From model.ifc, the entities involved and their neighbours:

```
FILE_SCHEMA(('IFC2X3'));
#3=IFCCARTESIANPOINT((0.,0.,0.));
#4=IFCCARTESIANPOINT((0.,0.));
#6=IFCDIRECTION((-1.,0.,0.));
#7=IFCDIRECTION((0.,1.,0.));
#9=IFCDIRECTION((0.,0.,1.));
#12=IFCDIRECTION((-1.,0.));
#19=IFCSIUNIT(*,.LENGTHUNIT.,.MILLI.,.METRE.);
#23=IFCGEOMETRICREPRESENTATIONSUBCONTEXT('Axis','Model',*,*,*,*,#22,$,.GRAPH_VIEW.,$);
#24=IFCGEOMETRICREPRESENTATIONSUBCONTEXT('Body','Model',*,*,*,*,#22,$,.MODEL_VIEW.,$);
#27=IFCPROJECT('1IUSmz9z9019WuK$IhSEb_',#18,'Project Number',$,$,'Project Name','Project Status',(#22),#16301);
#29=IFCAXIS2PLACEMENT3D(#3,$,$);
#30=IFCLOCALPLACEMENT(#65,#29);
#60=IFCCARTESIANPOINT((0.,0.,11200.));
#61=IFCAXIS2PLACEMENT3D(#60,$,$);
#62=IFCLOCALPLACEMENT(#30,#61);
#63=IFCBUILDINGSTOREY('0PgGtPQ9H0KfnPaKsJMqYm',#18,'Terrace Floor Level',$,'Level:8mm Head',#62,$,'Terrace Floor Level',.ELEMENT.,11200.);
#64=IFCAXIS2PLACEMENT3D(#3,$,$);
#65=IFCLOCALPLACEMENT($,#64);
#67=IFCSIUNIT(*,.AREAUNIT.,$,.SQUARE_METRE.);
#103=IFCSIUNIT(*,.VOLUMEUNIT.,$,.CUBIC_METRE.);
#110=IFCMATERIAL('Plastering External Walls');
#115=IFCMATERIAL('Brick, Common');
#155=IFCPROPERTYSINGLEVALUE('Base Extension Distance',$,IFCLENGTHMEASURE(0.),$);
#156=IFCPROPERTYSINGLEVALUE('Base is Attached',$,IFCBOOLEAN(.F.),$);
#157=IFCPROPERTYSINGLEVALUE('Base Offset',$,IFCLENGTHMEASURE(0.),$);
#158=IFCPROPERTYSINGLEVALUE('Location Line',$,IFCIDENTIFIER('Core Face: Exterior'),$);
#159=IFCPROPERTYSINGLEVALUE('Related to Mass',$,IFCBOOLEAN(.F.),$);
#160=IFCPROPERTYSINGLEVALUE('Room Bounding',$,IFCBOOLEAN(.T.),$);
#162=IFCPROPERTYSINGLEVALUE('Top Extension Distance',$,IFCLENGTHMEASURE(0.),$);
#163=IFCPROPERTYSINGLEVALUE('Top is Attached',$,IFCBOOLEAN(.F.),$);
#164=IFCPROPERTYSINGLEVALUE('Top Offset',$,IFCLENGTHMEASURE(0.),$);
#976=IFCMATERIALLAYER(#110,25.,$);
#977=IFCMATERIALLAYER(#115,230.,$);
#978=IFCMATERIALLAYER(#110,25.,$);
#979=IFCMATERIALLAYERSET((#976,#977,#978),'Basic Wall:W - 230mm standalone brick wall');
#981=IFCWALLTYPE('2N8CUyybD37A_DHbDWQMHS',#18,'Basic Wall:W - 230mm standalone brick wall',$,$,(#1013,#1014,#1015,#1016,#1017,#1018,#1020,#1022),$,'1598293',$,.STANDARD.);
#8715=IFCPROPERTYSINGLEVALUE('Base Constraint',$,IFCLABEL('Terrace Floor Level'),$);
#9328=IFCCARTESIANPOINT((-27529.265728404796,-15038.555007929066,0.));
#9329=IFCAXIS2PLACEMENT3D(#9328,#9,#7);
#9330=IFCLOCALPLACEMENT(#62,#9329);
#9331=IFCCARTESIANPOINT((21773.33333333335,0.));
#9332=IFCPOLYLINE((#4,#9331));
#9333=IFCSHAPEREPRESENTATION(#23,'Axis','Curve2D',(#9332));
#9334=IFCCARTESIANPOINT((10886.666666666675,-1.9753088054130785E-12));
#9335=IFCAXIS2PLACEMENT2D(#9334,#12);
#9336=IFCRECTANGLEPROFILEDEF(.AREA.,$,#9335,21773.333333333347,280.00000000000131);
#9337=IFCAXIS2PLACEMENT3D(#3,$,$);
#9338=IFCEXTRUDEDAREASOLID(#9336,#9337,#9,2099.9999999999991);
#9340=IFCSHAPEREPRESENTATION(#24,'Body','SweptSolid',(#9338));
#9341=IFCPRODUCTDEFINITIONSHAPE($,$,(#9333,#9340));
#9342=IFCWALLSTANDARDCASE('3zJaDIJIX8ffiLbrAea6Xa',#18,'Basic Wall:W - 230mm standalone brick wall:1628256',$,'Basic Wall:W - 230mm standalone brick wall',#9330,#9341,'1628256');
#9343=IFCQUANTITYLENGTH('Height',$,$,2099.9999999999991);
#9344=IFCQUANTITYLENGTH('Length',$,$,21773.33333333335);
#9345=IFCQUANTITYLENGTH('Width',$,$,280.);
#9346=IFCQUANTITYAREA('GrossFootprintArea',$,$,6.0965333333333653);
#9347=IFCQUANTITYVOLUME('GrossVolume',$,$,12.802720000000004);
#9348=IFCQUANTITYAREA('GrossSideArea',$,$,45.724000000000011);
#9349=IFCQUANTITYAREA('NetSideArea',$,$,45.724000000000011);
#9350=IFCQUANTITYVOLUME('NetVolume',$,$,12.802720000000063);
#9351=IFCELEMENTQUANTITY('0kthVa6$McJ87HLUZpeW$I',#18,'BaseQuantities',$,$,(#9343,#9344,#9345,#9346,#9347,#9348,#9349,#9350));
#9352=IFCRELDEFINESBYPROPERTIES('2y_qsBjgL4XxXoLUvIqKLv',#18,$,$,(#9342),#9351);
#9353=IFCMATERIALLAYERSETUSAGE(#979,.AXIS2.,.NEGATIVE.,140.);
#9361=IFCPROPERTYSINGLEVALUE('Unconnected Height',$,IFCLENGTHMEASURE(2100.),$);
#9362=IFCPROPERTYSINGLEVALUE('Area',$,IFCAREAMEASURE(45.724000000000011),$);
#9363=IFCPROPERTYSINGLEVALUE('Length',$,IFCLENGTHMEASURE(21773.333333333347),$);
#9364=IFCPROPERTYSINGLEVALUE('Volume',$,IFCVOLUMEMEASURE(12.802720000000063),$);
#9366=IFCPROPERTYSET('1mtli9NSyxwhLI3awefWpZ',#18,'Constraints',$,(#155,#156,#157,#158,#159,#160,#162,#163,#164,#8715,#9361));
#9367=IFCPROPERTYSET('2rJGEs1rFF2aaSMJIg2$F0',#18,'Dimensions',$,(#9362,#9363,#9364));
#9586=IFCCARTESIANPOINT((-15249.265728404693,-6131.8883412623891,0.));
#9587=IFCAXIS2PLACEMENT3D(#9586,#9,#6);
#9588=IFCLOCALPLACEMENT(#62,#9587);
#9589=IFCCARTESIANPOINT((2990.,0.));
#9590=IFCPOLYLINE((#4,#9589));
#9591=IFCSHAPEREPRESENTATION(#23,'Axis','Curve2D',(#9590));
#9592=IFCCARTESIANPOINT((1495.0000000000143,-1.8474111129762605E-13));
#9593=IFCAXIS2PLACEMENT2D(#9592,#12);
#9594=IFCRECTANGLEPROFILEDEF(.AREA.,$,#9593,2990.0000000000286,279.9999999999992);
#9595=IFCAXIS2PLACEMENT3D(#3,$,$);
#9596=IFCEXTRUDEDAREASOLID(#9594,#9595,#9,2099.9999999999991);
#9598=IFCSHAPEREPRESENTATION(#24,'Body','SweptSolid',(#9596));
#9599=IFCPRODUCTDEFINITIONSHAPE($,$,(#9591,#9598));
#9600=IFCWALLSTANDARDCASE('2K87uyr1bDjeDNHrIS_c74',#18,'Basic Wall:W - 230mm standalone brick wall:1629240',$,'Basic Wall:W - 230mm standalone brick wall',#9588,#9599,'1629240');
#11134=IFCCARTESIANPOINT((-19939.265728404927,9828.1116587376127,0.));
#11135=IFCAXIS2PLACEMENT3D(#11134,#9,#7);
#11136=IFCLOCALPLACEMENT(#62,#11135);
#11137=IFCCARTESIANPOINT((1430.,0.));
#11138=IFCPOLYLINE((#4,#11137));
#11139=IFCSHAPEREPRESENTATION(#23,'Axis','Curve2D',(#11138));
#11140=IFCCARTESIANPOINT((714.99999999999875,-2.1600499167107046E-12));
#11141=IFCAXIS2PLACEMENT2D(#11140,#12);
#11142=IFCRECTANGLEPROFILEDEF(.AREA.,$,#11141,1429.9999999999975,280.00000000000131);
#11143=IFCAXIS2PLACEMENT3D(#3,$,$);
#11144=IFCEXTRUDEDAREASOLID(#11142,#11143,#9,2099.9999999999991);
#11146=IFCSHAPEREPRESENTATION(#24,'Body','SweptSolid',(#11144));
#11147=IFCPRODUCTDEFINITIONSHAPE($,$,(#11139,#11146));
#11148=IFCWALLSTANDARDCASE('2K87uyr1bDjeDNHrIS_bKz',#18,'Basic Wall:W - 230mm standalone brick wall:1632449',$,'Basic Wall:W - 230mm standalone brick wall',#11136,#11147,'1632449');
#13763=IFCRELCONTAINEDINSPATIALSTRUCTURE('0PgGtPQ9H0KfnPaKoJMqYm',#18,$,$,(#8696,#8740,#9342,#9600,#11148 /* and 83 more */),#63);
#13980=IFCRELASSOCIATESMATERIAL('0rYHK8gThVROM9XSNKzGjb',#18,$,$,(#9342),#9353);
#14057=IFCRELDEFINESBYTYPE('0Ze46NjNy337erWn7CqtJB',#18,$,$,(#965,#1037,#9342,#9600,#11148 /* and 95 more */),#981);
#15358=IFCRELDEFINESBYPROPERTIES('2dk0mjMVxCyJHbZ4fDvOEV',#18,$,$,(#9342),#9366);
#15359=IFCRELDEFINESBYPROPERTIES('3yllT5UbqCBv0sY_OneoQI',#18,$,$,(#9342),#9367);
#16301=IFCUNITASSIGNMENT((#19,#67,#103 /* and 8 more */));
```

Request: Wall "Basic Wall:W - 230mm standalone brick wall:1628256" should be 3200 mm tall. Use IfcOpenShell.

```python
import ifcopenshell
import ifcopenshell.api.pset
import ifcopenshell.geom
import ifcopenshell.util.element
import ifcopenshell.util.representation
import ifcopenshell.util.shape
import ifcopenshell.util.unit

model = ifcopenshell.open("model.ifc")
unit_scale = ifcopenshell.util.unit.calculate_unit_scale(model)
area_scale = ifcopenshell.util.unit.calculate_unit_scale(model, "AREAUNIT")
volume_scale = ifcopenshell.util.unit.calculate_unit_scale(model, "VOLUMEUNIT")
settings = ifcopenshell.geom.settings()


def volume(element):
    """Net volume in cubic metres, openings subtracted."""
    shape = ifcopenshell.geom.create_shape(settings, element)
    return ifcopenshell.util.shape.get_volume(shape.geometry)


wall = model.by_guid("3zJaDIJIX8ffiLbrAea6Xa")
before = volume(wall)

body = ifcopenshell.util.representation.get_representation(wall, "Model", "Body")
solid = body.Items[0]
old_height = solid.Depth
solid.Depth = 3.2 / unit_scale
after = volume(wall)
thickness = 0.28  # wall thickness in metres

# Update the stored height, areas and volumes.
qto = model.by_id(ifcopenshell.util.element.get_pset(wall, "BaseQuantities", should_inherit=False)["id"])
ifcopenshell.api.pset.edit_qto(model, qto=qto, properties={
    "Height": solid.Depth,
    "GrossVolume": ifcopenshell.util.element.get_pset(wall, "BaseQuantities", "GrossVolume") * solid.Depth / old_height,
    "GrossSideArea": ifcopenshell.util.element.get_pset(wall, "BaseQuantities", "GrossSideArea") * solid.Depth / old_height,
    "NetSideArea": after / thickness / area_scale,
    "NetVolume": after / volume_scale,
})
pset = model.by_id(ifcopenshell.util.element.get_pset(wall, "Constraints", should_inherit=False)["id"])
ifcopenshell.api.pset.edit_pset(model, pset=pset, properties={
    "Unconnected Height": model.create_entity("IfcLengthMeasure", solid.Depth),
})
pset = model.by_id(ifcopenshell.util.element.get_pset(wall, "Dimensions", should_inherit=False)["id"])
ifcopenshell.api.pset.edit_pset(model, pset=pset, properties={
    "Area": model.create_entity("IfcAreaMeasure", after / thickness / area_scale),
    "Volume": model.create_entity("IfcVolumeMeasure", after / volume_scale),
})

print(f"height {old_height:g} -> {solid.Depth:g}, volume {before:.3f} -> {after:.3f} m3")

model.write("model_v2.ifc")
```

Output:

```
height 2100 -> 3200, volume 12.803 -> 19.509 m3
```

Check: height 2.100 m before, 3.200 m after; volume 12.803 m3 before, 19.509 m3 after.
